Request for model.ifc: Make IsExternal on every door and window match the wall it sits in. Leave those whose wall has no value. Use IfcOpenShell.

First a look at what the model holds.

```python
import ifcopenshell
import ifcopenshell.util.element

model = ifcopenshell.open("model.ifc")
print(model.schema)
seen = {}
for e in model.by_type("IfcDoor") + model.by_type("IfcWindow"):
    if not e.FillsVoids:
        continue
    host = e.FillsVoids[0].RelatingOpeningElement.VoidsElements[0].RelatingBuildingElement
    own = ifcopenshell.util.element.get_pset(e, f"Pset_{e.is_a()[3:].removesuffix('StandardCase')}Common", "IsExternal")
    wall = ifcopenshell.util.element.get_pset(host, "Pset_WallCommon", "IsExternal")
    seen[e.is_a(), own, wall] = seen.get((e.is_a(), own, wall), 0) + 1
for (cls, own, wall), count in sorted(seen.items(), key=str):
    print(count, cls, "IsExternal:", own, "| host wall:", wall)
```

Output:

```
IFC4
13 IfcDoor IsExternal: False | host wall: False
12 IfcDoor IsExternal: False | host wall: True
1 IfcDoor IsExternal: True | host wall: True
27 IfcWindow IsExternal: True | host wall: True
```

```python
import ifcopenshell
import ifcopenshell.api.pset
import ifcopenshell.util.element

model = ifcopenshell.open("model.ifc")

count = 0
for ifc_class, pset_name in (("IfcDoor", "Pset_DoorCommon"), ("IfcWindow", "Pset_WindowCommon")):
    for e in model.by_type(ifc_class):
        if not e.FillsVoids:
            continue
        host = e.FillsVoids[0].RelatingOpeningElement.VoidsElements[0].RelatingBuildingElement
        external = ifcopenshell.util.element.get_pset(host, "Pset_WallCommon", "IsExternal")
        if external is None or ifcopenshell.util.element.get_pset(e, pset_name, "IsExternal") == external:
            continue
        pset = ifcopenshell.api.pset.add_pset(model, product=e, name=pset_name)
        ifcopenshell.api.pset.edit_pset(model, pset=pset, properties={"IsExternal": external})
        count += 1

print(count, "updated")

model.write("model_edited.ifc")
```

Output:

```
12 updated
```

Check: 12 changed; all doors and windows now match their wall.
